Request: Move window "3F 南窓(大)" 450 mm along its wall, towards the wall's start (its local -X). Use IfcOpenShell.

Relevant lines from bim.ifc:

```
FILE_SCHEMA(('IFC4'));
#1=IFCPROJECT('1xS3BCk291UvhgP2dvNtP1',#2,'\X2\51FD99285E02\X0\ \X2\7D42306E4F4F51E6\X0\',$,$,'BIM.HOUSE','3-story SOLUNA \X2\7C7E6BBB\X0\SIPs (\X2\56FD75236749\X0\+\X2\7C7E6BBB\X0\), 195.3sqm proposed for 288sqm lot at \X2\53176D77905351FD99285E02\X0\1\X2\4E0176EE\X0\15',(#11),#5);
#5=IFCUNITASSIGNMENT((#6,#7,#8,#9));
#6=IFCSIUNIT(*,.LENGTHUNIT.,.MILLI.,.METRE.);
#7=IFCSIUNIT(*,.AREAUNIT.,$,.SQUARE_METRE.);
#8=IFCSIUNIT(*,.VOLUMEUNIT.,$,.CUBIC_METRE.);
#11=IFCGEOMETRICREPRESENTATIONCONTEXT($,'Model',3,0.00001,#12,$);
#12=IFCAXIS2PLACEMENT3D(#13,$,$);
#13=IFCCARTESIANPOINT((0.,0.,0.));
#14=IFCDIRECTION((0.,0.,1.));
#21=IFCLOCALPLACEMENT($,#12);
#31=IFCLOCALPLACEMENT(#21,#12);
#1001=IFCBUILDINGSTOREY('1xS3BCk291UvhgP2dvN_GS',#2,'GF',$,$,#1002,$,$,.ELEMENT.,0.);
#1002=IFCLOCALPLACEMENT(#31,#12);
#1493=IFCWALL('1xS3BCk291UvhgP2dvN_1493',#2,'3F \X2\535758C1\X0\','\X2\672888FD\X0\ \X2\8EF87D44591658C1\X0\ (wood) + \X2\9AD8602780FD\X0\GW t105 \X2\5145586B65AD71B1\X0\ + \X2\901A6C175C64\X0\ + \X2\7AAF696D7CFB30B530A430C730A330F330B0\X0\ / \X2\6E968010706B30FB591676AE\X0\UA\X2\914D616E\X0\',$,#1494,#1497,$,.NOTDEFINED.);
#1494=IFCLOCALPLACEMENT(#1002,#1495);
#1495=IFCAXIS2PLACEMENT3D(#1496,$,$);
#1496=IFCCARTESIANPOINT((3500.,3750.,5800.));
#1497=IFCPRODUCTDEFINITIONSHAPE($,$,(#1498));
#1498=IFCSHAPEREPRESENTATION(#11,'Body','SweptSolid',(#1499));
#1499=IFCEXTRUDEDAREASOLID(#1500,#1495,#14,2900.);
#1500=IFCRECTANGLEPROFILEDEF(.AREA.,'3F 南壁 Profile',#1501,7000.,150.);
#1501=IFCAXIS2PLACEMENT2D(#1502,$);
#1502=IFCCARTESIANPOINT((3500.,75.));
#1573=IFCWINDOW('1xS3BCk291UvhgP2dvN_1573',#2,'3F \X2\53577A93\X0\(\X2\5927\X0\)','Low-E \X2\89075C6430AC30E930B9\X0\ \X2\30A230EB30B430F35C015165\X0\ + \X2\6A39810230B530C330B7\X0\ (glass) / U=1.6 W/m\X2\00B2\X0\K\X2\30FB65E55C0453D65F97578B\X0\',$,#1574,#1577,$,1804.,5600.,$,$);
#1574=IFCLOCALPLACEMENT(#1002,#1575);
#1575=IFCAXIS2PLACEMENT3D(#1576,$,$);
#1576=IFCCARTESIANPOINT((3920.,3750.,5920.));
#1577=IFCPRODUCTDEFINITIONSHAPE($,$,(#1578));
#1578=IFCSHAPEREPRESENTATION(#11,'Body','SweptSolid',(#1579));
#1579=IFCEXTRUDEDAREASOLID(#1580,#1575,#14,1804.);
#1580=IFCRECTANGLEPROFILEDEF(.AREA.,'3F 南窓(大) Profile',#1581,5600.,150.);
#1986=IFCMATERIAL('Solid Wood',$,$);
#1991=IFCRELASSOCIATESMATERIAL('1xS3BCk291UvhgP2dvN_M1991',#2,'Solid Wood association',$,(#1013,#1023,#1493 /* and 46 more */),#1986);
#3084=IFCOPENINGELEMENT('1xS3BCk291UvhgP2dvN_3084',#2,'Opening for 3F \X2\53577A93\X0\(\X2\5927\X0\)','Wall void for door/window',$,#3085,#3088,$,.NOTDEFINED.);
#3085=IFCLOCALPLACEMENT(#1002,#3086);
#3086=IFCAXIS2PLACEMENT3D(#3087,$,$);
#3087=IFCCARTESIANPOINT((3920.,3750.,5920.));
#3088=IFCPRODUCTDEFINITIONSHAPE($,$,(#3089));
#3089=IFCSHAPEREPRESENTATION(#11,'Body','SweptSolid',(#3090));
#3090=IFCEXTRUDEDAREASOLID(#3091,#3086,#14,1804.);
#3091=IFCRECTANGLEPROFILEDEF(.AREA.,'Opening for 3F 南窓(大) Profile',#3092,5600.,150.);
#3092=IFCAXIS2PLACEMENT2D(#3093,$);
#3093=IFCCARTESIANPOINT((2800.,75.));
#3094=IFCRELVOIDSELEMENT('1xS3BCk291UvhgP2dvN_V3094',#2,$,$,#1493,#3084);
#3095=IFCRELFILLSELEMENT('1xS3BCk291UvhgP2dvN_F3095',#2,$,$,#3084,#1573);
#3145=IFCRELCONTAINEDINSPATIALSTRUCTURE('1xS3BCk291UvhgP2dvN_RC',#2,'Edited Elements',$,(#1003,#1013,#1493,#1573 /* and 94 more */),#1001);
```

```python
import ifcopenshell
import ifcopenshell.api.geometry
import ifcopenshell.util.placement

model = ifcopenshell.open("bim.ifc")

window = model.by_guid("1xS3BCk291UvhgP2dvN_1573")
opening = window.FillsVoids[0].RelatingOpeningElement
wall = opening.VoidsElements[0].RelatingBuildingElement

wall_matrix = ifcopenshell.util.placement.get_local_placement(wall.ObjectPlacement)
shift = wall_matrix[:3, 0] * -450.0
before = ifcopenshell.util.placement.get_local_placement(window.ObjectPlacement)[:3, 3].copy()

# The window is not placed relative to its opening, so move both.
for product in (opening, window):
    matrix = ifcopenshell.util.placement.get_local_placement(product.ObjectPlacement)
    matrix[:3, 3] += shift
    ifcopenshell.api.geometry.edit_object_placement(model, product=product, matrix=matrix, is_si=False)

after = ifcopenshell.util.placement.get_local_placement(window.ObjectPlacement)[:3, 3]
print("window moved by", (after - before).round(3) + 0.0)

model.write("bim_v2.ifc")
```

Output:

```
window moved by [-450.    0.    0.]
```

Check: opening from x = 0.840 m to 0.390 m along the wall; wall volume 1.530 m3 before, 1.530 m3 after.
